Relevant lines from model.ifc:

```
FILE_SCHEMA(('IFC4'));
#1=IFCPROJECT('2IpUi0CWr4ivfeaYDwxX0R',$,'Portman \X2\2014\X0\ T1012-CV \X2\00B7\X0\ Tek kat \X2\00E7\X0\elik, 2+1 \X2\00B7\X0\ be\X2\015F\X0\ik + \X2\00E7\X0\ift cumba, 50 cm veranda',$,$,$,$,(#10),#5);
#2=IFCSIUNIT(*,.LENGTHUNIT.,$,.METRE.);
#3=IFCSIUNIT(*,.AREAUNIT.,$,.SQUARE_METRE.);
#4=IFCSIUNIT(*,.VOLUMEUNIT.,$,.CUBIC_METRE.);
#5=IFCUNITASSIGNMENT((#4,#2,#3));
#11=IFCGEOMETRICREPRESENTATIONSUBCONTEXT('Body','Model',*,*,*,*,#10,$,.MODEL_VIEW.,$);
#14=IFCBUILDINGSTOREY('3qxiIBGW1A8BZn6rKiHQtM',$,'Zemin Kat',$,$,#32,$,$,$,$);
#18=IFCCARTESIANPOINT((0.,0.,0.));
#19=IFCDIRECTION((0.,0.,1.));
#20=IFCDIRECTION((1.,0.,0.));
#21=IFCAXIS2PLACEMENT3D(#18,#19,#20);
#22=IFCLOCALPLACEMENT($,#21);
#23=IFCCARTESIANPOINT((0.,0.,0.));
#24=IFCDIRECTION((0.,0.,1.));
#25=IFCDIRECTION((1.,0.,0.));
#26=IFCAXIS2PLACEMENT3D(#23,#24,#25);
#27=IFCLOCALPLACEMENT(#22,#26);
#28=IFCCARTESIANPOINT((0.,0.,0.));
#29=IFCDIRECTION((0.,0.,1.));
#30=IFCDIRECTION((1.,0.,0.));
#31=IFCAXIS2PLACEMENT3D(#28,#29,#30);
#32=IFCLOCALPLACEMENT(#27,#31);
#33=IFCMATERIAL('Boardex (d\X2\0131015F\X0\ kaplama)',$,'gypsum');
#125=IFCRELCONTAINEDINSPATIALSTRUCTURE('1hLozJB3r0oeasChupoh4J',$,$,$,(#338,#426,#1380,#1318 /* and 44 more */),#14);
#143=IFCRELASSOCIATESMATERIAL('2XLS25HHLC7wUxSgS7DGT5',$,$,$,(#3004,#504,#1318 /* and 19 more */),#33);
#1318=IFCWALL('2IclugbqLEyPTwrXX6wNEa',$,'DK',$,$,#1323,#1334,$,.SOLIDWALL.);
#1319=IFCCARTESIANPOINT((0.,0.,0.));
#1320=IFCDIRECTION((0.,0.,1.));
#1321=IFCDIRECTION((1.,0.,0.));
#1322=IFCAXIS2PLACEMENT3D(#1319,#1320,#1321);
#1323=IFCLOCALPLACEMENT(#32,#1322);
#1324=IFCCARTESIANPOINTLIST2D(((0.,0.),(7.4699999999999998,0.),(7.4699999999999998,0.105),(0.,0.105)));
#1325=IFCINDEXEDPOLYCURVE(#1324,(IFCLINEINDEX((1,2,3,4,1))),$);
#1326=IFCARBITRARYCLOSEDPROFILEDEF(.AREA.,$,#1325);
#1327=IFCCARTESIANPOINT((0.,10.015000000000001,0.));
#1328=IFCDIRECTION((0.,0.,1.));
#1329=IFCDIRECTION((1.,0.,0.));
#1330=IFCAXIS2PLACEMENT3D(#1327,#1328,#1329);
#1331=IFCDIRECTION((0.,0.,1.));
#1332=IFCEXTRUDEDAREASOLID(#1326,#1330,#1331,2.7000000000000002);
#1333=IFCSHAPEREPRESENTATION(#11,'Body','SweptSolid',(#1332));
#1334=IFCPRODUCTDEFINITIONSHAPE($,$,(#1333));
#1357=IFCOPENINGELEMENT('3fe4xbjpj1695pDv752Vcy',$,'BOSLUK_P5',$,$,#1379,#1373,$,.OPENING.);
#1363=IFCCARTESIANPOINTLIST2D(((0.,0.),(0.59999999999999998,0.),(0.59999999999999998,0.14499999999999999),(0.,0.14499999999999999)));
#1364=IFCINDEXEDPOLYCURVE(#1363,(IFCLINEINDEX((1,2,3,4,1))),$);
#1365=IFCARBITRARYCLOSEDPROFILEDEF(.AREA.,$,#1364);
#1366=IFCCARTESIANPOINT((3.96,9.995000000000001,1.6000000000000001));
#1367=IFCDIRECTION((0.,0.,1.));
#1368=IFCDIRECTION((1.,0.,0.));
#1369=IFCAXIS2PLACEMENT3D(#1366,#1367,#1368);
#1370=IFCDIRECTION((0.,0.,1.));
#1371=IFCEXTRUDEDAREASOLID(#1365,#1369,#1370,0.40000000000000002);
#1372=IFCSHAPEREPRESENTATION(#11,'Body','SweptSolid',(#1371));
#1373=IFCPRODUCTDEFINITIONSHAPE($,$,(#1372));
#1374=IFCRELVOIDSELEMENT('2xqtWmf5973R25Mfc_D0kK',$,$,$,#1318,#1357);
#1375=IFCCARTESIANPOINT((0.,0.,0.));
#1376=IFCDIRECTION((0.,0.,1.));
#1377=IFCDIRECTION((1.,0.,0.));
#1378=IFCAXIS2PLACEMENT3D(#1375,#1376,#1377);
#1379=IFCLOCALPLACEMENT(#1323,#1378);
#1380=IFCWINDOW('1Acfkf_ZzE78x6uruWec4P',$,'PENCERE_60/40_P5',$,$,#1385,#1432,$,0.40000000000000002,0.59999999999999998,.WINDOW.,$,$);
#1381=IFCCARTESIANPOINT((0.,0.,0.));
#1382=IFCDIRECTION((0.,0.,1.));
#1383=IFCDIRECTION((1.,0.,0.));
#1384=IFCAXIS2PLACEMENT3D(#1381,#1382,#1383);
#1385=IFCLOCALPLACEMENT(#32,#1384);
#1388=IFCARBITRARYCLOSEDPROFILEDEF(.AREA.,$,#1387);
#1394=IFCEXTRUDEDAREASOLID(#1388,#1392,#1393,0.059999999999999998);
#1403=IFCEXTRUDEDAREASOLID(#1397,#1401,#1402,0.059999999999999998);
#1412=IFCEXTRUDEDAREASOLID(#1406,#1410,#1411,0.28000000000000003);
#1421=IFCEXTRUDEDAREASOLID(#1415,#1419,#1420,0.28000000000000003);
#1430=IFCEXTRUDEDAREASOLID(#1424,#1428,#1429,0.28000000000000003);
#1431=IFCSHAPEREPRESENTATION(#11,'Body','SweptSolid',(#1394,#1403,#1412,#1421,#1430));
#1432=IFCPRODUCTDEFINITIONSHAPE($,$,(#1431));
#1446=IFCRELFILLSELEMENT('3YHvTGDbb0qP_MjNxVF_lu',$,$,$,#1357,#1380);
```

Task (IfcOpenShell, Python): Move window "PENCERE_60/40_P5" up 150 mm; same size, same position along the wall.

```python
import numpy as np
import ifcopenshell
import ifcopenshell.api.geometry
import ifcopenshell.util.placement
import ifcopenshell.util.unit

model = ifcopenshell.open("model.ifc")
unit_scale = ifcopenshell.util.unit.calculate_unit_scale(model)

window = model.by_guid("1Acfkf_ZzE78x6uruWec4P")
opening = window.FillsVoids[0].RelatingOpeningElement
dz = 0.15

shift = np.array([0.0, 0.0, dz])
# The window is not placed relative to its opening, so move both.
for product in (opening, window):
    matrix = ifcopenshell.util.placement.get_local_placement(product.ObjectPlacement)
    matrix[:3, 3] += shift
    ifcopenshell.api.geometry.edit_object_placement(model, product=product, matrix=matrix, is_si=False)

print(f"moved by {dz * unit_scale:+.3f} m")

model.write("model-out.ifc")
```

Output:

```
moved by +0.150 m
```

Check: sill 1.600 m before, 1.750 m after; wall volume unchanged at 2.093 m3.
